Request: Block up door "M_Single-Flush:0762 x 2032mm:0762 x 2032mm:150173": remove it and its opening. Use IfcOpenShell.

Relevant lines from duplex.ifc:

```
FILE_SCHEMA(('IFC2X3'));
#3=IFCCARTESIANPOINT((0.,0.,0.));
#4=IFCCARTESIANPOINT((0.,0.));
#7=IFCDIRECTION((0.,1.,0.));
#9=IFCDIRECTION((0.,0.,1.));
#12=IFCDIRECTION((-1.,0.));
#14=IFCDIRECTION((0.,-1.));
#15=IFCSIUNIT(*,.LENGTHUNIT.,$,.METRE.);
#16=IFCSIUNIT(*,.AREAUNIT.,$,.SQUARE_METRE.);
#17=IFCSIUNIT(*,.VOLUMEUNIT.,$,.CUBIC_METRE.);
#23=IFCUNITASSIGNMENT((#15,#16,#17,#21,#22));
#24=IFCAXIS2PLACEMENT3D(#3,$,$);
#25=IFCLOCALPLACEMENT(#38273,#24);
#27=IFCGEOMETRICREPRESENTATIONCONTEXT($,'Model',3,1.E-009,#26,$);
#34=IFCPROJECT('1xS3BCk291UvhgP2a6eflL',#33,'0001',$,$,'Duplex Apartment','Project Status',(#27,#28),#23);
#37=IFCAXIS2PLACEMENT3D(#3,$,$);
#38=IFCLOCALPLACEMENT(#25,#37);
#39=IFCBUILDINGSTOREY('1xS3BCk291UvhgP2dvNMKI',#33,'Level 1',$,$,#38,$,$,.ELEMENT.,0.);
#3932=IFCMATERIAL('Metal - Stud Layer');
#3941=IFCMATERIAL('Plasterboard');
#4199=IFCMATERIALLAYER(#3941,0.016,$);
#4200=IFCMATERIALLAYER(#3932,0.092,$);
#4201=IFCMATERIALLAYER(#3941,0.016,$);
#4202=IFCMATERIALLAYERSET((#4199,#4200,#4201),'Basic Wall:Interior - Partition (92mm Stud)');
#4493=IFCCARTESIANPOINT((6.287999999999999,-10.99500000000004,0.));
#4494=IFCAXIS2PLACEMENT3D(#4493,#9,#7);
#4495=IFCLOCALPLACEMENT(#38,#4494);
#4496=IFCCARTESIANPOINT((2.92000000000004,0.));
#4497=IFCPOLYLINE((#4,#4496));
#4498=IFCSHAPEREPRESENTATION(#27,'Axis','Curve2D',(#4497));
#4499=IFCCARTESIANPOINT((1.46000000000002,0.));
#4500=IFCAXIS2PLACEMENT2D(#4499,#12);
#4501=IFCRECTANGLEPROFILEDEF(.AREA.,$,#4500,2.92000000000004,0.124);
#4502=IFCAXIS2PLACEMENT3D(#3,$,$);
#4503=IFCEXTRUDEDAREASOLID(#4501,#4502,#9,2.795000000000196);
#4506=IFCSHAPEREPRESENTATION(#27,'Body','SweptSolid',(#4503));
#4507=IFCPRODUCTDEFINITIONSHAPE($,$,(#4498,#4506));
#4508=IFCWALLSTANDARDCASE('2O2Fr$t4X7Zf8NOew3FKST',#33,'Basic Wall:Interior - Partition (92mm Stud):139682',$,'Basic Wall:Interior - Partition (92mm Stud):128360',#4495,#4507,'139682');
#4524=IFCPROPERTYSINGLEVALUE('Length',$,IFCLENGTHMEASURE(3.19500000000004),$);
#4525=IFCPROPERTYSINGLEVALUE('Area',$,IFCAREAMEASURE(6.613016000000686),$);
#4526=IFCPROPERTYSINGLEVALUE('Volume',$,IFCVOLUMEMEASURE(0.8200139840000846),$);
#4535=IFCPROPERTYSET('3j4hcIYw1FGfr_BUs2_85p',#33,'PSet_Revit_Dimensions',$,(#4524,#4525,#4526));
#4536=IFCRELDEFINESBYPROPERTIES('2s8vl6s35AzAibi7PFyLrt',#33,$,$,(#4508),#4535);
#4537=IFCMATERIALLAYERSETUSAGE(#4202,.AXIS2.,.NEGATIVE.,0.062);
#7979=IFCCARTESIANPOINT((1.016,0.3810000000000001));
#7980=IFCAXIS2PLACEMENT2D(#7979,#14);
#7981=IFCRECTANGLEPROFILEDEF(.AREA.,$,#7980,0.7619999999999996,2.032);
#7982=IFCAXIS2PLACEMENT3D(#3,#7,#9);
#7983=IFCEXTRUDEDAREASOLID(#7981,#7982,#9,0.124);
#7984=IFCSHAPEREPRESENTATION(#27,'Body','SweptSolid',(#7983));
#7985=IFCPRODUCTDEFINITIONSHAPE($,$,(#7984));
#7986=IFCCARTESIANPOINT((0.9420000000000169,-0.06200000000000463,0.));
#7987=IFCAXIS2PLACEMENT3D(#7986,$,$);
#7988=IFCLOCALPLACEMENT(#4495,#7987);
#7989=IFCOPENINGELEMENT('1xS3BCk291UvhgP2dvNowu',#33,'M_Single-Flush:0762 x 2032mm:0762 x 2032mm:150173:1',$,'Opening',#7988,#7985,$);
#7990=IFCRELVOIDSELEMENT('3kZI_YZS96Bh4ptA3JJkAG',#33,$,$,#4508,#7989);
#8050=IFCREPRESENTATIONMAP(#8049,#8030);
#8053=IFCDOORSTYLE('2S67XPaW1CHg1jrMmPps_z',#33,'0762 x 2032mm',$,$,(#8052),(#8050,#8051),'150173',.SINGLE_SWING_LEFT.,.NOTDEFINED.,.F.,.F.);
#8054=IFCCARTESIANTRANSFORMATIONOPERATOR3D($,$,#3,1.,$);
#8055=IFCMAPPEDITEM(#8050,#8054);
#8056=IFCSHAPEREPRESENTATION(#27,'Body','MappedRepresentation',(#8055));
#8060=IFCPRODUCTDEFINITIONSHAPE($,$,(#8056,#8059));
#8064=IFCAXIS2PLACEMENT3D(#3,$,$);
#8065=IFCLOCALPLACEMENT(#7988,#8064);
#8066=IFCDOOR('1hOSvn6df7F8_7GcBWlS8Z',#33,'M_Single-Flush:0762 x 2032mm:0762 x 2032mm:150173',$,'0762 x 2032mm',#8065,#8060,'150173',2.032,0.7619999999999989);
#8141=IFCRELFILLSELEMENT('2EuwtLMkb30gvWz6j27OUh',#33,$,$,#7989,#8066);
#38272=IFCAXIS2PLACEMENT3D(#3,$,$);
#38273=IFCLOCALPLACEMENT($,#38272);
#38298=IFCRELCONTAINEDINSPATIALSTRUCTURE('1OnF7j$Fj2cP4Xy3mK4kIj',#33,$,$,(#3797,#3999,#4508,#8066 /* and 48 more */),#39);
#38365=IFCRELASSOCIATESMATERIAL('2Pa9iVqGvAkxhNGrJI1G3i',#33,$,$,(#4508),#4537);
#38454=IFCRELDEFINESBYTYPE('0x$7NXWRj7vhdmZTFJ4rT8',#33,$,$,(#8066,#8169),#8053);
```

```python
import ifcopenshell
import ifcopenshell.api.feature
import ifcopenshell.api.pset
import ifcopenshell.api.root
import ifcopenshell.geom
import ifcopenshell.util.element
import ifcopenshell.util.shape
import ifcopenshell.util.unit

model = ifcopenshell.open("duplex.ifc")
area_scale = ifcopenshell.util.unit.calculate_unit_scale(model, "AREAUNIT")
volume_scale = ifcopenshell.util.unit.calculate_unit_scale(model, "VOLUMEUNIT")
settings = ifcopenshell.geom.settings()


def volume(element):
    """Net volume in cubic metres, openings subtracted."""
    shape = ifcopenshell.geom.create_shape(settings, element)
    return ifcopenshell.util.shape.get_volume(shape.geometry)


door = model.by_guid("1hOSvn6df7F8_7GcBWlS8Z")
opening = door.FillsVoids[0].RelatingOpeningElement
wall = opening.VoidsElements[0].RelatingBuildingElement
before = volume(wall)

ifcopenshell.api.root.remove_product(model, product=door)
ifcopenshell.api.feature.remove_feature(model, feature=opening)

after = volume(wall)
thickness = 0.124  # wall thickness in metres

# Update the wall's stored quantities.
pset = model.by_id(ifcopenshell.util.element.get_pset(wall, "PSet_Revit_Dimensions", should_inherit=False)["id"])
ifcopenshell.api.pset.edit_pset(model, pset=pset, properties={
    "Area": model.create_entity("IfcAreaMeasure", after / thickness / area_scale),
    "Volume": model.create_entity("IfcVolumeMeasure", after / volume_scale),
})

print(f"wall volume {before:.3f} -> {after:.3f} m3")

model.write("duplex-out.ifc")
```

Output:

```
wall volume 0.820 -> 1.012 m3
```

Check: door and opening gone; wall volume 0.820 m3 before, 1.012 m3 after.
